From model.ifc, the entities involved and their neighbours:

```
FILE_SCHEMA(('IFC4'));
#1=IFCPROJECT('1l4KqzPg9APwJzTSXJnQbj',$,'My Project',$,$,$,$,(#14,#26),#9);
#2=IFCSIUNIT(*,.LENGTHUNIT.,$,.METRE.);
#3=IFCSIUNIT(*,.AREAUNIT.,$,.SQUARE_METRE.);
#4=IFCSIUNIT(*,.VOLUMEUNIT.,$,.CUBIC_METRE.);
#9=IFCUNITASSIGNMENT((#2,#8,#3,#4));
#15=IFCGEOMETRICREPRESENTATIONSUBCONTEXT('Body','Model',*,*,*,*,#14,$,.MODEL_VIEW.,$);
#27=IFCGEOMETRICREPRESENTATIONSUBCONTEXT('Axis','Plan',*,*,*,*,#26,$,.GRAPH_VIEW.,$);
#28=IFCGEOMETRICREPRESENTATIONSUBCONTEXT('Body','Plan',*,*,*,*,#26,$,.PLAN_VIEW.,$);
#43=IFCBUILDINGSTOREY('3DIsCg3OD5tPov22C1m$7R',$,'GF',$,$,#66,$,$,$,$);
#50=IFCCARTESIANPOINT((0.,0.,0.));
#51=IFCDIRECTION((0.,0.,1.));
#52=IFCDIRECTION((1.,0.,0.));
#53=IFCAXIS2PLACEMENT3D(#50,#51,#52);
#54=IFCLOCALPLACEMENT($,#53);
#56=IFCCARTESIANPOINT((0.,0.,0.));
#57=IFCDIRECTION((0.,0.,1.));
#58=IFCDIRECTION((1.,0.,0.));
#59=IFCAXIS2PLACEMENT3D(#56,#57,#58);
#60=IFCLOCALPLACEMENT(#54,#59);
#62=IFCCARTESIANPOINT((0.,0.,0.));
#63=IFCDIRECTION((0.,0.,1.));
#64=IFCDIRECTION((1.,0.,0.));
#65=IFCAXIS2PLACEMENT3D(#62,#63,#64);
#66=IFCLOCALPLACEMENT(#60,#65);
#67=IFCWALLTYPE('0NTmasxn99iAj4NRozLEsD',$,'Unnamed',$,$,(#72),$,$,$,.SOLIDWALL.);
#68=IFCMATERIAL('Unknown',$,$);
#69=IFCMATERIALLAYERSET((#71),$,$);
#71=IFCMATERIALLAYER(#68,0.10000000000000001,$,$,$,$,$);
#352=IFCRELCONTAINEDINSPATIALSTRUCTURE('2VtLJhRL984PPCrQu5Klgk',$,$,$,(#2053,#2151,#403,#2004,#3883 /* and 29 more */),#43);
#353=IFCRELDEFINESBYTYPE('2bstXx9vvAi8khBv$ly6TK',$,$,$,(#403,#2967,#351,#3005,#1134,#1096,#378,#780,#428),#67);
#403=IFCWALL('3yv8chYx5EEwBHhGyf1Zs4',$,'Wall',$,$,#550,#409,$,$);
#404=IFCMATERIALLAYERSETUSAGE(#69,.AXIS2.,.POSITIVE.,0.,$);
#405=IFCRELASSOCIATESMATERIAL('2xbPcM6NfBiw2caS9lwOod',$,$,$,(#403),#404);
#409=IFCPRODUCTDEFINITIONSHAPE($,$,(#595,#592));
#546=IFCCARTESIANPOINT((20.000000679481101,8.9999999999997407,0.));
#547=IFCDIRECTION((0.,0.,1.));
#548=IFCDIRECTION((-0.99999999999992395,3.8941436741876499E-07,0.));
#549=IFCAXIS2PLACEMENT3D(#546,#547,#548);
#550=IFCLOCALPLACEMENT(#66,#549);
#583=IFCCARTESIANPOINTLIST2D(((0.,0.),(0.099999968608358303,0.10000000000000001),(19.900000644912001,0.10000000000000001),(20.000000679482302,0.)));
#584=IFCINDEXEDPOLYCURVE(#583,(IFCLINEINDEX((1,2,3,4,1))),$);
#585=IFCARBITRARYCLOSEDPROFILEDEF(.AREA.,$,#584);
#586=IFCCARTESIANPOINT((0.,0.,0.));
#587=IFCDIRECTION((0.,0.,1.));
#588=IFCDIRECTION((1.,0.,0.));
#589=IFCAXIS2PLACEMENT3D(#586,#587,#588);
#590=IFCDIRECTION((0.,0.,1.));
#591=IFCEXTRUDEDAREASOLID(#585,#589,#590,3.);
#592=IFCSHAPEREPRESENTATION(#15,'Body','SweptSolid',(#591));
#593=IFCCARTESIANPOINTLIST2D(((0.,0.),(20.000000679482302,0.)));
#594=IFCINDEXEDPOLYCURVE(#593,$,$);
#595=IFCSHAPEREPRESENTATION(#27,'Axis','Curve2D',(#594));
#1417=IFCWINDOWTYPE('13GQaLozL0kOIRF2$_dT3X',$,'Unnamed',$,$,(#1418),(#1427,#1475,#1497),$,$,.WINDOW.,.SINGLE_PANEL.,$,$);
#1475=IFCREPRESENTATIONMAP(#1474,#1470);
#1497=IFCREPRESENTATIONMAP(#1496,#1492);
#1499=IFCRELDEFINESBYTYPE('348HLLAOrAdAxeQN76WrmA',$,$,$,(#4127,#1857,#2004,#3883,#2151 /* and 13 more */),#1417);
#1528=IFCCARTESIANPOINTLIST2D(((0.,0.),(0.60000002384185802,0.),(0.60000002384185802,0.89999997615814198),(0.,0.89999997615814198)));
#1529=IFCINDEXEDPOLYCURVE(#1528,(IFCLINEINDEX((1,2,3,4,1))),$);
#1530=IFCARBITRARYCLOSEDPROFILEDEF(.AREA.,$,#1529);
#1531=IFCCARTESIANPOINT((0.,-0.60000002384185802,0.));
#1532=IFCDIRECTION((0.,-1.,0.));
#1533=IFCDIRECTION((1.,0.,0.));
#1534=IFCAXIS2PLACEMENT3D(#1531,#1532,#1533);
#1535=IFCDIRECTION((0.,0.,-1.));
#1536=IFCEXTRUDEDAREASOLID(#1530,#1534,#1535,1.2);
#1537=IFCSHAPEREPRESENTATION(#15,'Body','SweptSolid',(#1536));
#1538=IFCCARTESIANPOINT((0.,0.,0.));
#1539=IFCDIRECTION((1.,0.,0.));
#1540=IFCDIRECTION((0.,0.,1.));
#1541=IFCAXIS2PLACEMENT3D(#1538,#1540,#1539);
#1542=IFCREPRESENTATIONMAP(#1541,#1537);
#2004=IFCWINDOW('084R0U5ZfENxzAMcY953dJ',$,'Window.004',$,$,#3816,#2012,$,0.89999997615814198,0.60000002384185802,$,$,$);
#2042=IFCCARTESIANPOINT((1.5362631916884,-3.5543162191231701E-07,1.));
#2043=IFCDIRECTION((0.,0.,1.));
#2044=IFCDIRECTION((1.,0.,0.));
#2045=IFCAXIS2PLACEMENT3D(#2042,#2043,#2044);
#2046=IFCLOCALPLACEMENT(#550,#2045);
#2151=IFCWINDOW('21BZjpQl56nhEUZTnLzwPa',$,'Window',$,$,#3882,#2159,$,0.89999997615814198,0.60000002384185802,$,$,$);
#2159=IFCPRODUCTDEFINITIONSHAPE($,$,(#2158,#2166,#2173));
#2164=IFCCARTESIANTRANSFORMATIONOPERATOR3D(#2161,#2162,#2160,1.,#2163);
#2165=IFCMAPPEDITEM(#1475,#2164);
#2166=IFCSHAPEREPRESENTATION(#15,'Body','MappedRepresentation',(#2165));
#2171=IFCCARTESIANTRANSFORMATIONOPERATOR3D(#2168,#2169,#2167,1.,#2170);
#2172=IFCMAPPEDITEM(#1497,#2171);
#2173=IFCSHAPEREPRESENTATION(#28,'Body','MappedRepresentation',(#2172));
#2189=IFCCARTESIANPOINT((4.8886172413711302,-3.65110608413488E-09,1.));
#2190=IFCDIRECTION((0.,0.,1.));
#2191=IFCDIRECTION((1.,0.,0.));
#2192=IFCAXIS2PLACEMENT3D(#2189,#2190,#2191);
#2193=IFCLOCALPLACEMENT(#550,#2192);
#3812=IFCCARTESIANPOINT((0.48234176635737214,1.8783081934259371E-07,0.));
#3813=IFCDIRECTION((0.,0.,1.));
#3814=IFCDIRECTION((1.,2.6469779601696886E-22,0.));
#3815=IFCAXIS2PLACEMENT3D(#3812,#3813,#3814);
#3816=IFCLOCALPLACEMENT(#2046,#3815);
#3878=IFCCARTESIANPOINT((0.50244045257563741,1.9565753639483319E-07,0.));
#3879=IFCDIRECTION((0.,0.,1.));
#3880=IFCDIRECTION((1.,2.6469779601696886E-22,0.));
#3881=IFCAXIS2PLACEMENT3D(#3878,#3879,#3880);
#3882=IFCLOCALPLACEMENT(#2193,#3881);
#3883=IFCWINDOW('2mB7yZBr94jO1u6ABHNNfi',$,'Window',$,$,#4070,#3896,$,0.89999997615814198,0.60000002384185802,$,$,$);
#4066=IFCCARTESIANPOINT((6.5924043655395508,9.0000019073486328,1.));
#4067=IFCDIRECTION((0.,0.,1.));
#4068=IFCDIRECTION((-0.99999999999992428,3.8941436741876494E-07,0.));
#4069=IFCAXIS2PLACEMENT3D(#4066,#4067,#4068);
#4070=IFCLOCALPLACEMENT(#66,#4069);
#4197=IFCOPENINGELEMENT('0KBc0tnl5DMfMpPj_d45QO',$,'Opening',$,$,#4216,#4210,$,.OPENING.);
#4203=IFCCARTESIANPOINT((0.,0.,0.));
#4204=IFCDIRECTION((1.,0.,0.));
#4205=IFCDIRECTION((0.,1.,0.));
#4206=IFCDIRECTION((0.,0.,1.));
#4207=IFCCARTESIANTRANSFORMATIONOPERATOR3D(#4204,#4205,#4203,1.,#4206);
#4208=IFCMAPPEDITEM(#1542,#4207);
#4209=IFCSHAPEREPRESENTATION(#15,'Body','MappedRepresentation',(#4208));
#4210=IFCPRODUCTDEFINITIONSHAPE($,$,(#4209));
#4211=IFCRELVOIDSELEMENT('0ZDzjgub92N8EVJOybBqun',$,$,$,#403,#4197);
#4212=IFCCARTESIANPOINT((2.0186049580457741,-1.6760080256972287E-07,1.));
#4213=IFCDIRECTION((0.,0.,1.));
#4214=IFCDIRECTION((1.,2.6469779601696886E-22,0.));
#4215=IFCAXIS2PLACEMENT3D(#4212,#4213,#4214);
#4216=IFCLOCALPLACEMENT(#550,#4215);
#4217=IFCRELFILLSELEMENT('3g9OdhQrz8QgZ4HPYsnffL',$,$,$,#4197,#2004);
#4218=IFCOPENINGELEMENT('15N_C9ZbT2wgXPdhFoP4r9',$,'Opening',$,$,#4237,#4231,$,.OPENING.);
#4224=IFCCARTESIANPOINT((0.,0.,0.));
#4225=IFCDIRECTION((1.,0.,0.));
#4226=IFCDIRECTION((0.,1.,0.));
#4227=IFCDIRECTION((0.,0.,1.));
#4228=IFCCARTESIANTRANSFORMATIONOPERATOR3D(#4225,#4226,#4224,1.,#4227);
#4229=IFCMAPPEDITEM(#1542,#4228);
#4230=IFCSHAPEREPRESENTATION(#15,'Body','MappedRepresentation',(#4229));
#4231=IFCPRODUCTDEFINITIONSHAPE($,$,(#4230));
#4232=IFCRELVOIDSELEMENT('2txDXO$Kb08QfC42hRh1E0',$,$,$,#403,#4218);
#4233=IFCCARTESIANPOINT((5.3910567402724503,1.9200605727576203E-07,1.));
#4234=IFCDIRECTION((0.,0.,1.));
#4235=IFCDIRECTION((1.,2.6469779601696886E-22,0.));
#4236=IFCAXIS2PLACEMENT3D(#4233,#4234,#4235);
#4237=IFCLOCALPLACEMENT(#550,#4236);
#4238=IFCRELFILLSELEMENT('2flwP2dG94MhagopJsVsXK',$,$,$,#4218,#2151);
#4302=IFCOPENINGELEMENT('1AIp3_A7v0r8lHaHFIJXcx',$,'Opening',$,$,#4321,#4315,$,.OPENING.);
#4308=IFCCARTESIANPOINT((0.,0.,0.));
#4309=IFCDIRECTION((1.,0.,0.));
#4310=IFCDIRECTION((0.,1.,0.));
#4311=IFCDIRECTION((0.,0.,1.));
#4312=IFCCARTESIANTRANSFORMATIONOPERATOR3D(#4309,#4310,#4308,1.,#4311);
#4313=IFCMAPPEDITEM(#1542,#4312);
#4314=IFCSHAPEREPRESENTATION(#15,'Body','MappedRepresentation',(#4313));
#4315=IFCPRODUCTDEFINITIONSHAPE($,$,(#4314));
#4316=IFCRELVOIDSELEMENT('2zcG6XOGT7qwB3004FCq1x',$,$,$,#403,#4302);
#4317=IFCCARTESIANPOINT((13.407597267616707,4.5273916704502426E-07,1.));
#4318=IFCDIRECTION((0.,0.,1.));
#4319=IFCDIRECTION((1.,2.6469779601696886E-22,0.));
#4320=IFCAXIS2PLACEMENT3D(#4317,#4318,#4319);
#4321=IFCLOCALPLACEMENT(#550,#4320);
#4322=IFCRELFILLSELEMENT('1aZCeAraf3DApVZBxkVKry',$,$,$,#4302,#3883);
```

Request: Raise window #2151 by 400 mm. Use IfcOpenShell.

```python
import numpy as np
import ifcopenshell
import ifcopenshell.api.geometry
import ifcopenshell.util.placement
import ifcopenshell.util.unit

model = ifcopenshell.open("model.ifc")
unit_scale = ifcopenshell.util.unit.calculate_unit_scale(model)

window = model.by_guid("21BZjpQl56nhEUZTnLzwPa")
opening = window.FillsVoids[0].RelatingOpeningElement
dz = 0.4

shift = np.array([0.0, 0.0, dz])
# The window is not placed relative to its opening, so move both.
for product in (opening, window):
    matrix = ifcopenshell.util.placement.get_local_placement(product.ObjectPlacement)
    matrix[:3, 3] += shift
    ifcopenshell.api.geometry.edit_object_placement(model, product=product, matrix=matrix, is_si=False)

print(f"moved by {dz * unit_scale:+.3f} m")

model.write("model_edited.ifc")
```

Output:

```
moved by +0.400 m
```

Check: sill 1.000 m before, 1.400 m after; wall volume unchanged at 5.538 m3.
